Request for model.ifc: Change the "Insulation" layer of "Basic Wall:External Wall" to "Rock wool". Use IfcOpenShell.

First a look at what the model holds.

```python
import ifcopenshell
import ifcopenshell.util.element

model = ifcopenshell.open("model.ifc")
print(model.schema)
for layer_set in model.by_type("IfcMaterialLayerSet"):
    if layer_set.LayerSetName == "Basic Wall:External Wall":
        for layer in layer_set.MaterialLayers:
            print(layer.id(), layer.Material and layer.Material.Name, layer.LayerThickness, sep=" | ")
        print(len(ifcopenshell.util.element.get_elements_by_material(model, layer_set)), "elements and types use it")
print(sorted(m.Name for m in model.by_type("IfcMaterial") if m.Name)[:60])
```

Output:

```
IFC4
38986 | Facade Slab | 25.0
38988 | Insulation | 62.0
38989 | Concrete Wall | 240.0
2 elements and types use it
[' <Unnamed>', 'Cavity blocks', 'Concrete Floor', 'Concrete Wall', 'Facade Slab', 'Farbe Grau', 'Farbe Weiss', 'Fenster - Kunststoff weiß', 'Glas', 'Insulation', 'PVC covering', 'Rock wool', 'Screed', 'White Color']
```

```python
import ifcopenshell
import ifcopenshell.api.material

model = ifcopenshell.open("model.ifc")

layer_set = next(s for s in model.by_type("IfcMaterialLayerSet") if s.LayerSetName == "Basic Wall:External Wall")
layer = next(l for l in layer_set.MaterialLayers if l.Material and l.Material.Name == "Insulation")
material = next(m for m in model.by_type("IfcMaterial") if m.Name == "Rock wool")

# Point this one layer at the other material; renaming the old one would change it everywhere.
ifcopenshell.api.material.edit_layer(model, layer=layer, attributes={}, material=material)

print([l.Material.Name if l.Material else None for l in layer_set.MaterialLayers])

model.write("model_rev.ifc")
```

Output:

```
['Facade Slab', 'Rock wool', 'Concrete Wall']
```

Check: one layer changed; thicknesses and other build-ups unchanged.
